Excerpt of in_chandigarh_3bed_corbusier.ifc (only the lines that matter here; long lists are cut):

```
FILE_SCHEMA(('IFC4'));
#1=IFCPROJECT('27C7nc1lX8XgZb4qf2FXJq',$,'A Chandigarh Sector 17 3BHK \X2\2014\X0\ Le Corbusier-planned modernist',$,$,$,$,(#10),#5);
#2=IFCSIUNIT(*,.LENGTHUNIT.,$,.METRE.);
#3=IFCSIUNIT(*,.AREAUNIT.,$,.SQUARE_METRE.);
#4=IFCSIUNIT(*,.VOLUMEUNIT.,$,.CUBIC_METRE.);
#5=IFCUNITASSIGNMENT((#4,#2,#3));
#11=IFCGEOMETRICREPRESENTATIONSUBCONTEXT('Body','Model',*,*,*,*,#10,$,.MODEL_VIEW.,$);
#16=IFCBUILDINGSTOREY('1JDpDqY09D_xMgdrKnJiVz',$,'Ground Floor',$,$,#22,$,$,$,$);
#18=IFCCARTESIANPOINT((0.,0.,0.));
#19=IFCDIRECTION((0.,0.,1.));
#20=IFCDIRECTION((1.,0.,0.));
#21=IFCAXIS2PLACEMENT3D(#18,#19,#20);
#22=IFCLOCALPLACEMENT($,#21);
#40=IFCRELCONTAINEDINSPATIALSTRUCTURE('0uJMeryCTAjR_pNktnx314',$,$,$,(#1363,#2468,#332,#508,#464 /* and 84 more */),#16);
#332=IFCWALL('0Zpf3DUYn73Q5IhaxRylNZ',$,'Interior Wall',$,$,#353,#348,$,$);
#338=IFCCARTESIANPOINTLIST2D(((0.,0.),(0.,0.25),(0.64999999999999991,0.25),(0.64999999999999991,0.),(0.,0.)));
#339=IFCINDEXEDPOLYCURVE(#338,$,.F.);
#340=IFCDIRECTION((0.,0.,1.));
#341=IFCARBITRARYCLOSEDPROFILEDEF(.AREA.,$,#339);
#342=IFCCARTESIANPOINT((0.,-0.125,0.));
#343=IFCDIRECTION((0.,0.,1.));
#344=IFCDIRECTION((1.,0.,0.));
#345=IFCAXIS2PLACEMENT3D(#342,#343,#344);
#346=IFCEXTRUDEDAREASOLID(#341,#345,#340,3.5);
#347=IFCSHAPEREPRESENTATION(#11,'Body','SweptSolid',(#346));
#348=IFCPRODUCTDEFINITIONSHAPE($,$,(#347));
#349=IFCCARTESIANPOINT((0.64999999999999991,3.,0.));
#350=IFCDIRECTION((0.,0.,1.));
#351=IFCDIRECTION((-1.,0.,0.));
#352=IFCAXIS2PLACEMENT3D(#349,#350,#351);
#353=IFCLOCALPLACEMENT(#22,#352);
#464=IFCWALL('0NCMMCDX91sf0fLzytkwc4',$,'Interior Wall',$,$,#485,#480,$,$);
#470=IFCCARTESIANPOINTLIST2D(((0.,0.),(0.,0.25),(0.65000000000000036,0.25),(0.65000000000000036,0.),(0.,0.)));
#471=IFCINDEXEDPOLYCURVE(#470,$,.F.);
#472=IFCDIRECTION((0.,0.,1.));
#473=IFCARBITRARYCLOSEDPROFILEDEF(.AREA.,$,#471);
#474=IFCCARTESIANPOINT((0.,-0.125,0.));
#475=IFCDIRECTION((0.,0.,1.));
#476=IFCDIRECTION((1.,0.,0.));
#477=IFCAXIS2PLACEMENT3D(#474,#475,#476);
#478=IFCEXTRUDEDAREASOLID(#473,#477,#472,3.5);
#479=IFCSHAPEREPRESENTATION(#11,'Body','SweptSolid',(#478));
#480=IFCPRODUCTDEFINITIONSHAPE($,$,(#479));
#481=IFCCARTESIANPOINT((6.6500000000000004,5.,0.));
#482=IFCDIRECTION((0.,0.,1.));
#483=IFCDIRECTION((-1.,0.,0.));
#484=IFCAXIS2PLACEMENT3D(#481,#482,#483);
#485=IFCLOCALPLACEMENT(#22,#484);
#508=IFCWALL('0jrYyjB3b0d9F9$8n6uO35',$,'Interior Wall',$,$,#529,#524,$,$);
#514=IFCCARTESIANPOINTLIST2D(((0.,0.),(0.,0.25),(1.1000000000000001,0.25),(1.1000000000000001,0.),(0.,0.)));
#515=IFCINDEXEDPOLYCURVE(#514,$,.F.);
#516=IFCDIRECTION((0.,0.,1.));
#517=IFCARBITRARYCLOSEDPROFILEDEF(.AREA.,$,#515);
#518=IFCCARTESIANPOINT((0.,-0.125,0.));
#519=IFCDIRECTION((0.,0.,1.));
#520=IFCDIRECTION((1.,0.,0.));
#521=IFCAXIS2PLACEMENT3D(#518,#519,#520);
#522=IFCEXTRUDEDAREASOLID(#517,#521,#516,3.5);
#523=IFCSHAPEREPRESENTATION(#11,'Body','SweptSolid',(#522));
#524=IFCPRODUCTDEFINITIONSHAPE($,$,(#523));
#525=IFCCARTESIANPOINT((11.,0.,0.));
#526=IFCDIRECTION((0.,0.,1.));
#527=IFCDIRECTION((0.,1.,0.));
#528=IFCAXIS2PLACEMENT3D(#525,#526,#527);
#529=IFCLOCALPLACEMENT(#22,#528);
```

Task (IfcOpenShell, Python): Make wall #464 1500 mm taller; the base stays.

```python
import ifcopenshell
import ifcopenshell.geom
import ifcopenshell.util.representation
import ifcopenshell.util.shape
import ifcopenshell.util.unit

model = ifcopenshell.open("in_chandigarh_3bed_corbusier.ifc")
unit_scale = ifcopenshell.util.unit.calculate_unit_scale(model)
settings = ifcopenshell.geom.settings()


def volume(element):
    """Net volume in cubic metres, openings subtracted."""
    shape = ifcopenshell.geom.create_shape(settings, element)
    return ifcopenshell.util.shape.get_volume(shape.geometry)


wall = model.by_guid("0NCMMCDX91sf0fLzytkwc4")
before = volume(wall)

body = ifcopenshell.util.representation.get_representation(wall, "Model", "Body")
solid = body.Items[0]
old_height = solid.Depth
solid.Depth += 1.5 / unit_scale
after = volume(wall)

print(f"height {old_height:g} -> {solid.Depth:g}, volume {before:.3f} -> {after:.3f} m3")

model.write("in_chandigarh_3bed_corbusier_edited.ifc")
```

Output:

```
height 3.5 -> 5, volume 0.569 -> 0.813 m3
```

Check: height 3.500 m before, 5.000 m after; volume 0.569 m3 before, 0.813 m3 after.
